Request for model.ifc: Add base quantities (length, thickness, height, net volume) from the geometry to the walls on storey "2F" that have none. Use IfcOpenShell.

First a look at what the model holds.

```python
import ifcopenshell
import ifcopenshell.util.element
import ifcopenshell.util.unit

model = ifcopenshell.open("model.ifc")
print(model.schema)
for unit_type in ("LENGTHUNIT", "AREAUNIT", "VOLUMEUNIT"):
    print(unit_type, ifcopenshell.util.unit.calculate_unit_scale(model, unit_type))
storey = next(s for s in model.by_type("IfcBuildingStorey") if s.Name == "2F")
walls = [e for e in ifcopenshell.util.element.get_decomposition(storey) if e.is_a("IfcWall")]
for e in sorted(walls, key=lambda e: e.id()):
    print(e.id(), e.is_a(), e.Name, list(ifcopenshell.util.element.get_psets(e, qtos_only=True)), sep=" | ")
```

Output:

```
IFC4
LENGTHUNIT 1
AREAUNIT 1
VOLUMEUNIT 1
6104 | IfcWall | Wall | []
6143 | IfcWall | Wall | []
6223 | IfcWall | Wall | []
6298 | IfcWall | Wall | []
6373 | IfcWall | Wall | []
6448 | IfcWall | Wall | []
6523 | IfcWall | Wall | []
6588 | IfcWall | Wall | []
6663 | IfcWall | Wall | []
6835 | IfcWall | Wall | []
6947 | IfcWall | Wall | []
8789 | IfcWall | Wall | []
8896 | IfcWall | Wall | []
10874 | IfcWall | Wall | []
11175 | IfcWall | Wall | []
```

```python
import ifcopenshell
import ifcopenshell.api.pset
import ifcopenshell.geom
import ifcopenshell.util.element
import ifcopenshell.util.shape
import ifcopenshell.util.unit

model = ifcopenshell.open("model.ifc")
unit_scale = ifcopenshell.util.unit.calculate_unit_scale(model)
volume_scale = ifcopenshell.util.unit.calculate_unit_scale(model, "VOLUMEUNIT")
settings = ifcopenshell.geom.settings()

storey = next(s for s in model.by_type("IfcBuildingStorey") if s.Name == "2F")
walls = [e for e in ifcopenshell.util.element.get_decomposition(storey) if e.is_a("IfcWall")]

for e in sorted(walls, key=lambda e: e.id()):
    if ifcopenshell.util.element.get_psets(e, qtos_only=True, should_inherit=False):
        continue
    # Geometry comes back in metres, in the element's own axes.
    shape = ifcopenshell.geom.create_shape(settings, e)
    values = {
        "Length": ifcopenshell.util.shape.get_x(shape.geometry) / unit_scale,
        "Width": ifcopenshell.util.shape.get_y(shape.geometry) / unit_scale,
        "Height": ifcopenshell.util.shape.get_z(shape.geometry) / unit_scale,
        "NetVolume": ifcopenshell.util.shape.get_volume(shape.geometry) / volume_scale,
    }
    qto = ifcopenshell.api.pset.add_qto(model, product=e, name="Qto_WallBaseQuantities")
    ifcopenshell.api.pset.edit_qto(model, qto=qto, properties=values)
    print(e.id(), {k: round(v, 3) for k, v in values.items()})

model.write("model_edited.ifc")
```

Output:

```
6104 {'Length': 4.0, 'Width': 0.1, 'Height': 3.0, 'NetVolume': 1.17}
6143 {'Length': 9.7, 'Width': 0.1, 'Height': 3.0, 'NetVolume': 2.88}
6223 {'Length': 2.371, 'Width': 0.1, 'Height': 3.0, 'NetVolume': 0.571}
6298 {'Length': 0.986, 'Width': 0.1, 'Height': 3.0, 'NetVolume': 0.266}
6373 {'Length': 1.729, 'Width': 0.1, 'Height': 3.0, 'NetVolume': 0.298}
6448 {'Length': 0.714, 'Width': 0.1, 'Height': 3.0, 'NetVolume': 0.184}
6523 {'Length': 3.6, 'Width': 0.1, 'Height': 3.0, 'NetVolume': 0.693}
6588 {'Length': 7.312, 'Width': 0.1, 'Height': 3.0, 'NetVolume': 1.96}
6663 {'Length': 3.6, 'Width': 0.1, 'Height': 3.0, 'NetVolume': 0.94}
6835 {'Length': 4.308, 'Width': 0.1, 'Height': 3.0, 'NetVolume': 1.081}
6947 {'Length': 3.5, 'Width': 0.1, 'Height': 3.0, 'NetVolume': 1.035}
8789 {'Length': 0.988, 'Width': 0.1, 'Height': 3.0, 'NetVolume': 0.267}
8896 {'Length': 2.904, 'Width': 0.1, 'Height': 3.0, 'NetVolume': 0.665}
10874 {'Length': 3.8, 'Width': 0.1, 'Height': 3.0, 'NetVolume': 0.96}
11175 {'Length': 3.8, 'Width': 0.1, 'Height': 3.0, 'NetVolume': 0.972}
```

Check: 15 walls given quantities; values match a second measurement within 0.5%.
